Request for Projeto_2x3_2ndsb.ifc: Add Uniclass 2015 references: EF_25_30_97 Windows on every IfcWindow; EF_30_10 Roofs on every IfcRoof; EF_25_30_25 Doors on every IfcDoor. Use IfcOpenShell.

First a look at what the model holds.

```python
import ifcopenshell

model = ifcopenshell.open("Projeto_2x3_2ndsb.ifc")
print(model.schema)
print("classifications:", [c.Name for c in model.by_type("IfcClassification")])
for ifc_class in ("IfcDoor", "IfcRoof", "IfcStair", "IfcWall", "IfcWindow"):
    print(ifc_class, len(model.by_type(ifc_class)))
```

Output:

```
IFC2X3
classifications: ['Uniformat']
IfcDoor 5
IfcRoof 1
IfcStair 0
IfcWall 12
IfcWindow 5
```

```python
import ifcopenshell
import ifcopenshell.api.classification

model = ifcopenshell.open("Projeto_2x3_2ndsb.ifc")

# IFC2X3 requires Source and Edition and has no link from the project to the system.
system = model.create_entity("IfcClassification", Source="NBS", Edition="2015", Name="Uniclass 2015")

codes = {
    "IfcWindow": ("EF_25_30_97", "Windows"),
    "IfcRoof": ("EF_30_10", "Roofs"),
    "IfcDoor": ("EF_25_30_25", "Doors"),
}
for ifc_class, (code, name) in codes.items():
    products = model.by_type(ifc_class)
    ifcopenshell.api.classification.add_reference(
        model, products=products, classification=system, identification=code, name=name
    )
    print(code, len(products))

model.write("Projeto_2x3_2ndsb_rev.ifc")
```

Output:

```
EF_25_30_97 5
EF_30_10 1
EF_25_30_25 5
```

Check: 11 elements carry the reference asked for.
